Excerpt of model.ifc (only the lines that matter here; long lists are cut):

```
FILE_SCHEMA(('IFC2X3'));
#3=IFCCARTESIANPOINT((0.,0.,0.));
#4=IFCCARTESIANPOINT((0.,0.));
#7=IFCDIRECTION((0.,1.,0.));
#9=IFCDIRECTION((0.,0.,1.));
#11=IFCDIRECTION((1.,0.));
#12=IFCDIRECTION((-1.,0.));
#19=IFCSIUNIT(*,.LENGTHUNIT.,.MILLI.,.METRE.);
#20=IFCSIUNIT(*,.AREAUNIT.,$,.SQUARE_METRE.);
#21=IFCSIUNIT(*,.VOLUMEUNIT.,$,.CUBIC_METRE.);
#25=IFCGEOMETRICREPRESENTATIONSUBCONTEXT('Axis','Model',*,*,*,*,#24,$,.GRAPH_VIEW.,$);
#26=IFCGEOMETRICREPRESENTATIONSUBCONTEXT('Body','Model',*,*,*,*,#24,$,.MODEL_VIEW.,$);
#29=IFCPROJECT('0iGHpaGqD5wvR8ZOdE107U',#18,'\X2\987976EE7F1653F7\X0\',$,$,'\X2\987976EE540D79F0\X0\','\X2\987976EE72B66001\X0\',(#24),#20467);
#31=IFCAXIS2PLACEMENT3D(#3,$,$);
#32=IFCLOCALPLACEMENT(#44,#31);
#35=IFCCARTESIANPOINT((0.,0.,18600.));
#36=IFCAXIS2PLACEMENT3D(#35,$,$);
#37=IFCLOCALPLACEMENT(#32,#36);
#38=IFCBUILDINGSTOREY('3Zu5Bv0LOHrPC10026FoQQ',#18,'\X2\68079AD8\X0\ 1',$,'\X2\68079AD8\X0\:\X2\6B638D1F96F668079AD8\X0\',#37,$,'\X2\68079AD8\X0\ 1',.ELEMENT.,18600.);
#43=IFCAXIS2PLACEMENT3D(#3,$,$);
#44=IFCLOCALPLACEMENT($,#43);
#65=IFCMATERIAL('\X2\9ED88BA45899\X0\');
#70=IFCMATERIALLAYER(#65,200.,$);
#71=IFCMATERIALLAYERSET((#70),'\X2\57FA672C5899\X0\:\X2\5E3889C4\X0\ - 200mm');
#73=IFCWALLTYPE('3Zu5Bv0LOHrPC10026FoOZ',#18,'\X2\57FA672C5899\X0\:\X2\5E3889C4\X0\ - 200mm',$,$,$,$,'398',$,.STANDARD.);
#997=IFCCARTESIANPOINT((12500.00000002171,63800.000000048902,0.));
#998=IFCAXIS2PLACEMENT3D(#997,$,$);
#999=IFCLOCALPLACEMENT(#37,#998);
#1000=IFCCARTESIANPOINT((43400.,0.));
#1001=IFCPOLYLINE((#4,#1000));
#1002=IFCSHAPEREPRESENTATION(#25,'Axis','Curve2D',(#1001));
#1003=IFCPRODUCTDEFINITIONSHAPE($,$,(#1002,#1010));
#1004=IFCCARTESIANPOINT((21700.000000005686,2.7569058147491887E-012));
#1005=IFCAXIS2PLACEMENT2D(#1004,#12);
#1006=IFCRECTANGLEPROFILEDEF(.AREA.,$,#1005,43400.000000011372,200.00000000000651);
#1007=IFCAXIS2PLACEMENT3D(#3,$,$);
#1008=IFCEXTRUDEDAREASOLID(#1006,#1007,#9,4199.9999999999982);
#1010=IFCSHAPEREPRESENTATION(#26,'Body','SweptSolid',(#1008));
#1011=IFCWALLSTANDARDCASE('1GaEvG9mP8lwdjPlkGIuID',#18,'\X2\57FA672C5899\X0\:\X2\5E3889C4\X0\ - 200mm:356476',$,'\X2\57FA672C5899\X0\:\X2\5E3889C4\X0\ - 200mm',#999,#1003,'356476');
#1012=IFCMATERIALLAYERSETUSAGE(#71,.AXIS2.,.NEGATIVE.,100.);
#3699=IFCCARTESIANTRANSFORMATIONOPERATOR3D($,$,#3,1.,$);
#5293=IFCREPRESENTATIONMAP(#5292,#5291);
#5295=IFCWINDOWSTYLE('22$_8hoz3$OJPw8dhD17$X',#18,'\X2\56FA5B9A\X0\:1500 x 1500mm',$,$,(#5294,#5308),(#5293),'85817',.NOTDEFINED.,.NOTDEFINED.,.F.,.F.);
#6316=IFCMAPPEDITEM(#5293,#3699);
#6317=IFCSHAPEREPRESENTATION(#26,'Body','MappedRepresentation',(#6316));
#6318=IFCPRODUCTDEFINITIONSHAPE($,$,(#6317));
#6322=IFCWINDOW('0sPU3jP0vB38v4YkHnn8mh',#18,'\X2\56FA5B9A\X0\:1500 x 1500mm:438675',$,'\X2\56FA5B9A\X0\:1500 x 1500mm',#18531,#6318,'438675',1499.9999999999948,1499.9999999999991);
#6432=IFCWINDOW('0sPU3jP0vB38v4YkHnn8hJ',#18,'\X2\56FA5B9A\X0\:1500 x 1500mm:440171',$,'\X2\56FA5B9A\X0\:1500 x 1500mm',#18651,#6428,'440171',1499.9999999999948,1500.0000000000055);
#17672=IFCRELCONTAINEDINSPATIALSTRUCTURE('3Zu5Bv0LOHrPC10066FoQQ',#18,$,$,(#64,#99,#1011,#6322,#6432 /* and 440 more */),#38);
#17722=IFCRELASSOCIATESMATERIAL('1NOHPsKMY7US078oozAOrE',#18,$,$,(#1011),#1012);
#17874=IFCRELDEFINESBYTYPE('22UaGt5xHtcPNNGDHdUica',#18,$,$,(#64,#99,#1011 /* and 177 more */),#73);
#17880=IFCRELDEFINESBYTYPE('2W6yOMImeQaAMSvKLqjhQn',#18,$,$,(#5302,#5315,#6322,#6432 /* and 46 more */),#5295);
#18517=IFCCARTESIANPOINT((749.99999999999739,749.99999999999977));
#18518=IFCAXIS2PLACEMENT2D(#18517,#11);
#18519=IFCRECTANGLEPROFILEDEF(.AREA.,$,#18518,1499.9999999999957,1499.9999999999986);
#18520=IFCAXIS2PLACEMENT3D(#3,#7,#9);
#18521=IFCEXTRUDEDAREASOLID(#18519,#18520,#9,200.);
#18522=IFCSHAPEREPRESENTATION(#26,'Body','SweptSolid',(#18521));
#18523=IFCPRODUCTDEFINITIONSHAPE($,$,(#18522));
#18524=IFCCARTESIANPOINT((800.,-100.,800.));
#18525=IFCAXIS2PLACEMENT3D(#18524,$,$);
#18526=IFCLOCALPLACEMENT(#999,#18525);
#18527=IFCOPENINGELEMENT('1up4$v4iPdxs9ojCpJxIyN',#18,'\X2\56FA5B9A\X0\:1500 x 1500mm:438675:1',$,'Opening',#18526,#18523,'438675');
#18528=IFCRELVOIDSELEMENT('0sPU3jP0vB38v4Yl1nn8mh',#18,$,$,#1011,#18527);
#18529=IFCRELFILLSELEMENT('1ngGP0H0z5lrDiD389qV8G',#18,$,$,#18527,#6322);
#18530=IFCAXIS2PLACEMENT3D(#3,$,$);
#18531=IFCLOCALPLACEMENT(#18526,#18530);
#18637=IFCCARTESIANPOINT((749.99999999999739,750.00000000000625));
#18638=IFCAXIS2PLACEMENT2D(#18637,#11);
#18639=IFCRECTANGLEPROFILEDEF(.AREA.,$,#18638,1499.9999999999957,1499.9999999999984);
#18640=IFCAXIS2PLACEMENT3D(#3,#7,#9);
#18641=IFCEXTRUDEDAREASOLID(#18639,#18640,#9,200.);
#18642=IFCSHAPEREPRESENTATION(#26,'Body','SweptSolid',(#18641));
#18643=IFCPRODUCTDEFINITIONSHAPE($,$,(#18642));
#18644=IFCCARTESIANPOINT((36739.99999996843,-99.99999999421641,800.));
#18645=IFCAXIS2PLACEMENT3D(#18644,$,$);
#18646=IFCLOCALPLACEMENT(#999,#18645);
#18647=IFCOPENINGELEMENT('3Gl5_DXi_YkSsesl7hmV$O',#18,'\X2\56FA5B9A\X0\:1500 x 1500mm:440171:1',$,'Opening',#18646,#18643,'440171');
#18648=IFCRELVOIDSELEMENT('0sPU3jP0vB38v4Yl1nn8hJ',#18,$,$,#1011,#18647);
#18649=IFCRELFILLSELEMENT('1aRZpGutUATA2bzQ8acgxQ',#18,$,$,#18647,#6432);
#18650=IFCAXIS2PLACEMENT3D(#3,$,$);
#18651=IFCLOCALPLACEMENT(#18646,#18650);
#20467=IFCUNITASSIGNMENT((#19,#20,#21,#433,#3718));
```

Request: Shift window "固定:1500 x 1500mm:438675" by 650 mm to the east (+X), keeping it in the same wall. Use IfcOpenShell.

```python
import ifcopenshell
import ifcopenshell.api.geometry
import ifcopenshell.util.placement
import ifcopenshell.util.unit

model = ifcopenshell.open("model.ifc")
unit_scale = ifcopenshell.util.unit.calculate_unit_scale(model)

window = model.by_guid("0sPU3jP0vB38v4YkHnn8mh")
opening = window.FillsVoids[0].RelatingOpeningElement
wall = opening.VoidsElements[0].RelatingBuildingElement

wall_matrix = ifcopenshell.util.placement.get_local_placement(wall.ObjectPlacement)
shift = wall_matrix[:3, 0] * 0.65 / unit_scale
before = ifcopenshell.util.placement.get_local_placement(window.ObjectPlacement)[:3, 3].copy()

# The window is placed relative to its opening, so it follows when the opening moves.
matrix = ifcopenshell.util.placement.get_local_placement(opening.ObjectPlacement)
matrix[:3, 3] += shift
ifcopenshell.api.geometry.edit_object_placement(
    model, product=opening, matrix=matrix, is_si=False, should_transform_children=True
)

after = ifcopenshell.util.placement.get_local_placement(window.ObjectPlacement)[:3, 3]
print("window moved by", (after - before).round(3) + 0.0)

model.write("model_edited.ifc")
```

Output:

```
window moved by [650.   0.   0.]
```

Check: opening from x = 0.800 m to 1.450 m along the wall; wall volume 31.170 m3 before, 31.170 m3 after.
